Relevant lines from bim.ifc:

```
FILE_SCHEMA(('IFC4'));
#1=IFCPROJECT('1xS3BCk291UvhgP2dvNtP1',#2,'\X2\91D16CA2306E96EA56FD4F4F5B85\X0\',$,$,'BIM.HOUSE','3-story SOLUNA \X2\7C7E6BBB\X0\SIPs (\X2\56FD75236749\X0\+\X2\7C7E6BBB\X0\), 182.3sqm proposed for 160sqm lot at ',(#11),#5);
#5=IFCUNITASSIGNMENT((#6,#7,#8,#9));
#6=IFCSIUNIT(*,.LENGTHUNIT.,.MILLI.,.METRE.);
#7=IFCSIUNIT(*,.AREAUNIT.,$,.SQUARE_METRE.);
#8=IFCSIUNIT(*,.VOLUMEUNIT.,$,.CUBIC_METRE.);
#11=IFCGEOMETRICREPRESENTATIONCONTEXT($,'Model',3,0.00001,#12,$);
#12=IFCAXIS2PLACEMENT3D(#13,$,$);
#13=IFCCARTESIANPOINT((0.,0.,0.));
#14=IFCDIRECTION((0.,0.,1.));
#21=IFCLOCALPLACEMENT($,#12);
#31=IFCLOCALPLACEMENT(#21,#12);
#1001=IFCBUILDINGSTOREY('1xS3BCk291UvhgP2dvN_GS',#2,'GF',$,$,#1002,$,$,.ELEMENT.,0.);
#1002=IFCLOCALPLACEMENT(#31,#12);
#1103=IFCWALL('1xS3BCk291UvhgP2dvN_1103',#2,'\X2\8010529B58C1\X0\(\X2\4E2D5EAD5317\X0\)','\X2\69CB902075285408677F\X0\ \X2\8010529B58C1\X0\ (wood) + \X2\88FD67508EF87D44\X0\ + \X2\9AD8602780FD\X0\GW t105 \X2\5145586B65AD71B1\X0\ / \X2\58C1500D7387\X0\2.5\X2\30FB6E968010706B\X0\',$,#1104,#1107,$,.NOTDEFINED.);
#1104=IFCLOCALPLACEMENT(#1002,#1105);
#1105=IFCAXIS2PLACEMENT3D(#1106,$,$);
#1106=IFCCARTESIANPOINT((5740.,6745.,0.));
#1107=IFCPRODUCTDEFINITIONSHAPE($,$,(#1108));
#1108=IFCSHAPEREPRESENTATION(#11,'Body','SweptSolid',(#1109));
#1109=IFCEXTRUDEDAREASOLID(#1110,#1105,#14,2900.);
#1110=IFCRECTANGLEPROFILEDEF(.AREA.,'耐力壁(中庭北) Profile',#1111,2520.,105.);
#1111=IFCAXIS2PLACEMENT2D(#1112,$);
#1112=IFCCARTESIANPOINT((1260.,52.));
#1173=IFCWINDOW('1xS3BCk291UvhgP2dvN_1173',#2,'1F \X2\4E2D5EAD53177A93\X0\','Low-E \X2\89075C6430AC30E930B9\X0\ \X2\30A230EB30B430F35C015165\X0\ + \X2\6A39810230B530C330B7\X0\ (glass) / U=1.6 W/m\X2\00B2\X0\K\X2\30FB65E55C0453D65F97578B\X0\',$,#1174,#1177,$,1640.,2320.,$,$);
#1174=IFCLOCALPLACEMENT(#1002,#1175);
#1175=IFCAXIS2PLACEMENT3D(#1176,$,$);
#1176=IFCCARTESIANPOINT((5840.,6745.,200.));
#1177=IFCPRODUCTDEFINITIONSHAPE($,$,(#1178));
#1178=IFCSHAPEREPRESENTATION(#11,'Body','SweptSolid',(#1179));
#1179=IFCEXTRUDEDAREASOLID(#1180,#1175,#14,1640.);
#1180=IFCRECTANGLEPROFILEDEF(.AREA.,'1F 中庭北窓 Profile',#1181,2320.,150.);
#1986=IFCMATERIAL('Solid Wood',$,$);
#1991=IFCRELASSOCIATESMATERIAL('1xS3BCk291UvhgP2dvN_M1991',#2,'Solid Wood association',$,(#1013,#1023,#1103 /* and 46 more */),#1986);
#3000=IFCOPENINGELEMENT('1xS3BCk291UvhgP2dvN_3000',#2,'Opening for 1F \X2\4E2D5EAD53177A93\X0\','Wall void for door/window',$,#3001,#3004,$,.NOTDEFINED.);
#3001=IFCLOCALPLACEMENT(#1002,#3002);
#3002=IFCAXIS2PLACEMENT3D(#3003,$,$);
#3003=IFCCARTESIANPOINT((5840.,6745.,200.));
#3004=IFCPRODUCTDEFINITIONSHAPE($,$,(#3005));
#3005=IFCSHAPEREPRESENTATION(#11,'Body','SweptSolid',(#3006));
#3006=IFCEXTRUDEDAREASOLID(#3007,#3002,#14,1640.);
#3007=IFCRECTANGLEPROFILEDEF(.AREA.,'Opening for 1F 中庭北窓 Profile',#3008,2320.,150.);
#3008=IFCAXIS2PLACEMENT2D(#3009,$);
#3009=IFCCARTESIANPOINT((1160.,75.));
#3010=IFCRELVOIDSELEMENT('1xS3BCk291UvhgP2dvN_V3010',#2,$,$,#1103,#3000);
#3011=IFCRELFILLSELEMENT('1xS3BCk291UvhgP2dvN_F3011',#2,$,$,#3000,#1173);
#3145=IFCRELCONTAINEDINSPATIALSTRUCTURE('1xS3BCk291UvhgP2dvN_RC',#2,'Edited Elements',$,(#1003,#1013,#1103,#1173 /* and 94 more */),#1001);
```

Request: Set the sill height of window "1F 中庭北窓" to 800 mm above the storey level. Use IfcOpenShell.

```python
import numpy as np
import ifcopenshell
import ifcopenshell.api.geometry
import ifcopenshell.geom
import ifcopenshell.util.element
import ifcopenshell.util.placement
import ifcopenshell.util.shape
import ifcopenshell.util.unit

model = ifcopenshell.open("bim.ifc")
unit_scale = ifcopenshell.util.unit.calculate_unit_scale(model)

window = model.by_guid("1xS3BCk291UvhgP2dvN_1173")
opening = window.FillsVoids[0].RelatingOpeningElement
storey = ifcopenshell.util.element.get_container(window, ifc_class="IfcBuildingStorey")
level = ifcopenshell.util.placement.get_local_placement(storey.ObjectPlacement)[2, 3]

# The opening's origin need not be at the sill, so measure its lowest point.
shape = ifcopenshell.geom.create_shape(ifcopenshell.geom.settings(), opening)
bottom = ifcopenshell.util.shape.get_shape_bottom_elevation(shape, shape.geometry) / unit_scale
dz = level + 800.0 - bottom

shift = np.array([0.0, 0.0, dz])
# The window is not placed relative to its opening, so move both.
for product in (opening, window):
    matrix = ifcopenshell.util.placement.get_local_placement(product.ObjectPlacement)
    matrix[:3, 3] += shift
    ifcopenshell.api.geometry.edit_object_placement(model, product=product, matrix=matrix, is_si=False)

print(f"moved by {dz * unit_scale:+.3f} m")

model.write("bim_v2.ifc")
```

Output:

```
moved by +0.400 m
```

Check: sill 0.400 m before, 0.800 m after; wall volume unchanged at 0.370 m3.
